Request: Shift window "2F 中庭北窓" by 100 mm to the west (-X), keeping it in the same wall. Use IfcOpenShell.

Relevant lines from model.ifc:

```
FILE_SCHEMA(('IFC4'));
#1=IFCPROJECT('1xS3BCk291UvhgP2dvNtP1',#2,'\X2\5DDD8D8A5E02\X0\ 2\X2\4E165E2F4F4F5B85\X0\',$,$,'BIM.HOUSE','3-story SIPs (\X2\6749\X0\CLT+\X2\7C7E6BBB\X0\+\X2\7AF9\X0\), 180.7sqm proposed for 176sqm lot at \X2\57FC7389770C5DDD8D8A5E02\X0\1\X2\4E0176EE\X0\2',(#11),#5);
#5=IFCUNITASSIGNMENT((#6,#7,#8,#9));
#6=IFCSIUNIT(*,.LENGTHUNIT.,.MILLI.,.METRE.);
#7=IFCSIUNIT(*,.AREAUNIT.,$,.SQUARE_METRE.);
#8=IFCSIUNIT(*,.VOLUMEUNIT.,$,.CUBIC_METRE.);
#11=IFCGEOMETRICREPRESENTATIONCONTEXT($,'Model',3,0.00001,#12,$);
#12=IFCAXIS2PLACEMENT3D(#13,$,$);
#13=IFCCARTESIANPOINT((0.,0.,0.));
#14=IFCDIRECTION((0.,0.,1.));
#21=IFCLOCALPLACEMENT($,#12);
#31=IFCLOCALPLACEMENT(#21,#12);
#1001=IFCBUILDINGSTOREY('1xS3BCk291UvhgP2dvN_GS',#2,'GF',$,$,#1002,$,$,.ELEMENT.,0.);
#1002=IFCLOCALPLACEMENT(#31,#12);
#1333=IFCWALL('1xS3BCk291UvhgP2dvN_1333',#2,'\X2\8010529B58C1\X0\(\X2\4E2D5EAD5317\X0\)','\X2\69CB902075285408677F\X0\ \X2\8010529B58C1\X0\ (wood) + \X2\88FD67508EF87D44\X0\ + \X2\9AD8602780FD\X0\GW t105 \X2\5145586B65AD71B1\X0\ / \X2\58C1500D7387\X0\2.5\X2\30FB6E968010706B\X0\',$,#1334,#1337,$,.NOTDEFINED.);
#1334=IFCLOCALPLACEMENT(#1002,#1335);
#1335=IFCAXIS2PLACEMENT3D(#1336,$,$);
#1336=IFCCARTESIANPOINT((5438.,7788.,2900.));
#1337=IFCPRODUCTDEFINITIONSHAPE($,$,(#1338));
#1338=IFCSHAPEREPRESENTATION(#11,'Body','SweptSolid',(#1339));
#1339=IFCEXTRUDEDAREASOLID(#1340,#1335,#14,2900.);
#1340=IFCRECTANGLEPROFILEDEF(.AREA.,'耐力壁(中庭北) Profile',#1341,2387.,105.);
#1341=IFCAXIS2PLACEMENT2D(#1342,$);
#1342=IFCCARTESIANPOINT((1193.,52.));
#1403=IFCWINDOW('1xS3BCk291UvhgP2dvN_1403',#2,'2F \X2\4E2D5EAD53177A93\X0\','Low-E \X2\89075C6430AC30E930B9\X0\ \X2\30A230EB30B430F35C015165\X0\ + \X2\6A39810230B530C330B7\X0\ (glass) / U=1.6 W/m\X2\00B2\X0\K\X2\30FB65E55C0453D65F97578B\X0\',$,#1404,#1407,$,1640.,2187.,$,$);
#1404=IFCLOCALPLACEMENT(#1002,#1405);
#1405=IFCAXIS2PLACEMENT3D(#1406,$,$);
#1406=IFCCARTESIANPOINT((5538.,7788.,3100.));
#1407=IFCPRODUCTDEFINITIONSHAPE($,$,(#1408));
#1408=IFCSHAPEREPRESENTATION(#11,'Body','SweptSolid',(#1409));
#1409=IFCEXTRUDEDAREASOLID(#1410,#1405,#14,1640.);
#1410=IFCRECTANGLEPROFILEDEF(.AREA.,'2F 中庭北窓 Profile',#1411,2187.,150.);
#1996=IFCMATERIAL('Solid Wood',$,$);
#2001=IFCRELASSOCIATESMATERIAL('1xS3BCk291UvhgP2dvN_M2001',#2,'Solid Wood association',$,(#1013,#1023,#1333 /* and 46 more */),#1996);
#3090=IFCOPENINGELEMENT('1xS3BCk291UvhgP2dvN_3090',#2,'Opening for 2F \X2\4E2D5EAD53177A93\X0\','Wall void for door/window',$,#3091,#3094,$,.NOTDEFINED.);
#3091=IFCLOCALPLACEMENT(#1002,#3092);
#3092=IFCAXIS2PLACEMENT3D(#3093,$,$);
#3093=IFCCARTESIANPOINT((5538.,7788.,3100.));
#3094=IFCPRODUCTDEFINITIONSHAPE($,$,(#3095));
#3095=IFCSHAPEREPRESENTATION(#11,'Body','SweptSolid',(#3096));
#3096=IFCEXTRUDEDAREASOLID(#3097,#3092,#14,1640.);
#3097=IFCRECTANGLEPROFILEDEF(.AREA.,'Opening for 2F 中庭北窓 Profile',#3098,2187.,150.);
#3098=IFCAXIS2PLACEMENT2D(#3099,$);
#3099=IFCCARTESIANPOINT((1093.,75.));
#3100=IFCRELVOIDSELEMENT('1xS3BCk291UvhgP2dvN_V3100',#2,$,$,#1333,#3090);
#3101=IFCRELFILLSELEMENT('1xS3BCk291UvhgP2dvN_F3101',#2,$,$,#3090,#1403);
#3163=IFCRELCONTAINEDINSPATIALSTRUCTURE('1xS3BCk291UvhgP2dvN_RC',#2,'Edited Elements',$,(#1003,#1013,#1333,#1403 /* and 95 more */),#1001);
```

```python
import ifcopenshell
import ifcopenshell.api.geometry
import ifcopenshell.util.placement

model = ifcopenshell.open("model.ifc")

window = model.by_guid("1xS3BCk291UvhgP2dvN_1403")
opening = window.FillsVoids[0].RelatingOpeningElement
wall = opening.VoidsElements[0].RelatingBuildingElement

wall_matrix = ifcopenshell.util.placement.get_local_placement(wall.ObjectPlacement)
shift = wall_matrix[:3, 0] * -100.0
before = ifcopenshell.util.placement.get_local_placement(window.ObjectPlacement)[:3, 3].copy()

# The window is not placed relative to its opening, so move both.
for product in (opening, window):
    matrix = ifcopenshell.util.placement.get_local_placement(product.ObjectPlacement)
    matrix[:3, 3] += shift
    ifcopenshell.api.geometry.edit_object_placement(model, product=product, matrix=matrix, is_si=False)

after = ifcopenshell.util.placement.get_local_placement(window.ObjectPlacement)[:3, 3]
print("window moved by", (after - before).round(3) + 0.0)

model.write("model_v2.ifc")
```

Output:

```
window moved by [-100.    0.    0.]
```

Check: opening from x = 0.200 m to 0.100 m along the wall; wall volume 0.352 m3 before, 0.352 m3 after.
